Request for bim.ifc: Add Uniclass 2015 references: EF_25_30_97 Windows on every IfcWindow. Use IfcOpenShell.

First a look at what the model holds.

```python
import ifcopenshell

model = ifcopenshell.open("bim.ifc")
print(model.schema)
print("classifications:", [c.Name for c in model.by_type("IfcClassification")])
for ifc_class in ("IfcDoor", "IfcRoof", "IfcStair", "IfcWall", "IfcWindow"):
    print(ifc_class, len(model.by_type(ifc_class)))
```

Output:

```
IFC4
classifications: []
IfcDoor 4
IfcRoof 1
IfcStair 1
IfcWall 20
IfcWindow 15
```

```python
import ifcopenshell
import ifcopenshell.api.classification

model = ifcopenshell.open("bim.ifc")

system = ifcopenshell.api.classification.add_classification(model, classification="Uniclass 2015")

codes = {
    "IfcWindow": ("EF_25_30_97", "Windows"),
}
for ifc_class, (code, name) in codes.items():
    products = model.by_type(ifc_class)
    ifcopenshell.api.classification.add_reference(
        model, products=products, classification=system, identification=code, name=name
    )
    print(code, len(products))

model.write("bim_v2.ifc")
```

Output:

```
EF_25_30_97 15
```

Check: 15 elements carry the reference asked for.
